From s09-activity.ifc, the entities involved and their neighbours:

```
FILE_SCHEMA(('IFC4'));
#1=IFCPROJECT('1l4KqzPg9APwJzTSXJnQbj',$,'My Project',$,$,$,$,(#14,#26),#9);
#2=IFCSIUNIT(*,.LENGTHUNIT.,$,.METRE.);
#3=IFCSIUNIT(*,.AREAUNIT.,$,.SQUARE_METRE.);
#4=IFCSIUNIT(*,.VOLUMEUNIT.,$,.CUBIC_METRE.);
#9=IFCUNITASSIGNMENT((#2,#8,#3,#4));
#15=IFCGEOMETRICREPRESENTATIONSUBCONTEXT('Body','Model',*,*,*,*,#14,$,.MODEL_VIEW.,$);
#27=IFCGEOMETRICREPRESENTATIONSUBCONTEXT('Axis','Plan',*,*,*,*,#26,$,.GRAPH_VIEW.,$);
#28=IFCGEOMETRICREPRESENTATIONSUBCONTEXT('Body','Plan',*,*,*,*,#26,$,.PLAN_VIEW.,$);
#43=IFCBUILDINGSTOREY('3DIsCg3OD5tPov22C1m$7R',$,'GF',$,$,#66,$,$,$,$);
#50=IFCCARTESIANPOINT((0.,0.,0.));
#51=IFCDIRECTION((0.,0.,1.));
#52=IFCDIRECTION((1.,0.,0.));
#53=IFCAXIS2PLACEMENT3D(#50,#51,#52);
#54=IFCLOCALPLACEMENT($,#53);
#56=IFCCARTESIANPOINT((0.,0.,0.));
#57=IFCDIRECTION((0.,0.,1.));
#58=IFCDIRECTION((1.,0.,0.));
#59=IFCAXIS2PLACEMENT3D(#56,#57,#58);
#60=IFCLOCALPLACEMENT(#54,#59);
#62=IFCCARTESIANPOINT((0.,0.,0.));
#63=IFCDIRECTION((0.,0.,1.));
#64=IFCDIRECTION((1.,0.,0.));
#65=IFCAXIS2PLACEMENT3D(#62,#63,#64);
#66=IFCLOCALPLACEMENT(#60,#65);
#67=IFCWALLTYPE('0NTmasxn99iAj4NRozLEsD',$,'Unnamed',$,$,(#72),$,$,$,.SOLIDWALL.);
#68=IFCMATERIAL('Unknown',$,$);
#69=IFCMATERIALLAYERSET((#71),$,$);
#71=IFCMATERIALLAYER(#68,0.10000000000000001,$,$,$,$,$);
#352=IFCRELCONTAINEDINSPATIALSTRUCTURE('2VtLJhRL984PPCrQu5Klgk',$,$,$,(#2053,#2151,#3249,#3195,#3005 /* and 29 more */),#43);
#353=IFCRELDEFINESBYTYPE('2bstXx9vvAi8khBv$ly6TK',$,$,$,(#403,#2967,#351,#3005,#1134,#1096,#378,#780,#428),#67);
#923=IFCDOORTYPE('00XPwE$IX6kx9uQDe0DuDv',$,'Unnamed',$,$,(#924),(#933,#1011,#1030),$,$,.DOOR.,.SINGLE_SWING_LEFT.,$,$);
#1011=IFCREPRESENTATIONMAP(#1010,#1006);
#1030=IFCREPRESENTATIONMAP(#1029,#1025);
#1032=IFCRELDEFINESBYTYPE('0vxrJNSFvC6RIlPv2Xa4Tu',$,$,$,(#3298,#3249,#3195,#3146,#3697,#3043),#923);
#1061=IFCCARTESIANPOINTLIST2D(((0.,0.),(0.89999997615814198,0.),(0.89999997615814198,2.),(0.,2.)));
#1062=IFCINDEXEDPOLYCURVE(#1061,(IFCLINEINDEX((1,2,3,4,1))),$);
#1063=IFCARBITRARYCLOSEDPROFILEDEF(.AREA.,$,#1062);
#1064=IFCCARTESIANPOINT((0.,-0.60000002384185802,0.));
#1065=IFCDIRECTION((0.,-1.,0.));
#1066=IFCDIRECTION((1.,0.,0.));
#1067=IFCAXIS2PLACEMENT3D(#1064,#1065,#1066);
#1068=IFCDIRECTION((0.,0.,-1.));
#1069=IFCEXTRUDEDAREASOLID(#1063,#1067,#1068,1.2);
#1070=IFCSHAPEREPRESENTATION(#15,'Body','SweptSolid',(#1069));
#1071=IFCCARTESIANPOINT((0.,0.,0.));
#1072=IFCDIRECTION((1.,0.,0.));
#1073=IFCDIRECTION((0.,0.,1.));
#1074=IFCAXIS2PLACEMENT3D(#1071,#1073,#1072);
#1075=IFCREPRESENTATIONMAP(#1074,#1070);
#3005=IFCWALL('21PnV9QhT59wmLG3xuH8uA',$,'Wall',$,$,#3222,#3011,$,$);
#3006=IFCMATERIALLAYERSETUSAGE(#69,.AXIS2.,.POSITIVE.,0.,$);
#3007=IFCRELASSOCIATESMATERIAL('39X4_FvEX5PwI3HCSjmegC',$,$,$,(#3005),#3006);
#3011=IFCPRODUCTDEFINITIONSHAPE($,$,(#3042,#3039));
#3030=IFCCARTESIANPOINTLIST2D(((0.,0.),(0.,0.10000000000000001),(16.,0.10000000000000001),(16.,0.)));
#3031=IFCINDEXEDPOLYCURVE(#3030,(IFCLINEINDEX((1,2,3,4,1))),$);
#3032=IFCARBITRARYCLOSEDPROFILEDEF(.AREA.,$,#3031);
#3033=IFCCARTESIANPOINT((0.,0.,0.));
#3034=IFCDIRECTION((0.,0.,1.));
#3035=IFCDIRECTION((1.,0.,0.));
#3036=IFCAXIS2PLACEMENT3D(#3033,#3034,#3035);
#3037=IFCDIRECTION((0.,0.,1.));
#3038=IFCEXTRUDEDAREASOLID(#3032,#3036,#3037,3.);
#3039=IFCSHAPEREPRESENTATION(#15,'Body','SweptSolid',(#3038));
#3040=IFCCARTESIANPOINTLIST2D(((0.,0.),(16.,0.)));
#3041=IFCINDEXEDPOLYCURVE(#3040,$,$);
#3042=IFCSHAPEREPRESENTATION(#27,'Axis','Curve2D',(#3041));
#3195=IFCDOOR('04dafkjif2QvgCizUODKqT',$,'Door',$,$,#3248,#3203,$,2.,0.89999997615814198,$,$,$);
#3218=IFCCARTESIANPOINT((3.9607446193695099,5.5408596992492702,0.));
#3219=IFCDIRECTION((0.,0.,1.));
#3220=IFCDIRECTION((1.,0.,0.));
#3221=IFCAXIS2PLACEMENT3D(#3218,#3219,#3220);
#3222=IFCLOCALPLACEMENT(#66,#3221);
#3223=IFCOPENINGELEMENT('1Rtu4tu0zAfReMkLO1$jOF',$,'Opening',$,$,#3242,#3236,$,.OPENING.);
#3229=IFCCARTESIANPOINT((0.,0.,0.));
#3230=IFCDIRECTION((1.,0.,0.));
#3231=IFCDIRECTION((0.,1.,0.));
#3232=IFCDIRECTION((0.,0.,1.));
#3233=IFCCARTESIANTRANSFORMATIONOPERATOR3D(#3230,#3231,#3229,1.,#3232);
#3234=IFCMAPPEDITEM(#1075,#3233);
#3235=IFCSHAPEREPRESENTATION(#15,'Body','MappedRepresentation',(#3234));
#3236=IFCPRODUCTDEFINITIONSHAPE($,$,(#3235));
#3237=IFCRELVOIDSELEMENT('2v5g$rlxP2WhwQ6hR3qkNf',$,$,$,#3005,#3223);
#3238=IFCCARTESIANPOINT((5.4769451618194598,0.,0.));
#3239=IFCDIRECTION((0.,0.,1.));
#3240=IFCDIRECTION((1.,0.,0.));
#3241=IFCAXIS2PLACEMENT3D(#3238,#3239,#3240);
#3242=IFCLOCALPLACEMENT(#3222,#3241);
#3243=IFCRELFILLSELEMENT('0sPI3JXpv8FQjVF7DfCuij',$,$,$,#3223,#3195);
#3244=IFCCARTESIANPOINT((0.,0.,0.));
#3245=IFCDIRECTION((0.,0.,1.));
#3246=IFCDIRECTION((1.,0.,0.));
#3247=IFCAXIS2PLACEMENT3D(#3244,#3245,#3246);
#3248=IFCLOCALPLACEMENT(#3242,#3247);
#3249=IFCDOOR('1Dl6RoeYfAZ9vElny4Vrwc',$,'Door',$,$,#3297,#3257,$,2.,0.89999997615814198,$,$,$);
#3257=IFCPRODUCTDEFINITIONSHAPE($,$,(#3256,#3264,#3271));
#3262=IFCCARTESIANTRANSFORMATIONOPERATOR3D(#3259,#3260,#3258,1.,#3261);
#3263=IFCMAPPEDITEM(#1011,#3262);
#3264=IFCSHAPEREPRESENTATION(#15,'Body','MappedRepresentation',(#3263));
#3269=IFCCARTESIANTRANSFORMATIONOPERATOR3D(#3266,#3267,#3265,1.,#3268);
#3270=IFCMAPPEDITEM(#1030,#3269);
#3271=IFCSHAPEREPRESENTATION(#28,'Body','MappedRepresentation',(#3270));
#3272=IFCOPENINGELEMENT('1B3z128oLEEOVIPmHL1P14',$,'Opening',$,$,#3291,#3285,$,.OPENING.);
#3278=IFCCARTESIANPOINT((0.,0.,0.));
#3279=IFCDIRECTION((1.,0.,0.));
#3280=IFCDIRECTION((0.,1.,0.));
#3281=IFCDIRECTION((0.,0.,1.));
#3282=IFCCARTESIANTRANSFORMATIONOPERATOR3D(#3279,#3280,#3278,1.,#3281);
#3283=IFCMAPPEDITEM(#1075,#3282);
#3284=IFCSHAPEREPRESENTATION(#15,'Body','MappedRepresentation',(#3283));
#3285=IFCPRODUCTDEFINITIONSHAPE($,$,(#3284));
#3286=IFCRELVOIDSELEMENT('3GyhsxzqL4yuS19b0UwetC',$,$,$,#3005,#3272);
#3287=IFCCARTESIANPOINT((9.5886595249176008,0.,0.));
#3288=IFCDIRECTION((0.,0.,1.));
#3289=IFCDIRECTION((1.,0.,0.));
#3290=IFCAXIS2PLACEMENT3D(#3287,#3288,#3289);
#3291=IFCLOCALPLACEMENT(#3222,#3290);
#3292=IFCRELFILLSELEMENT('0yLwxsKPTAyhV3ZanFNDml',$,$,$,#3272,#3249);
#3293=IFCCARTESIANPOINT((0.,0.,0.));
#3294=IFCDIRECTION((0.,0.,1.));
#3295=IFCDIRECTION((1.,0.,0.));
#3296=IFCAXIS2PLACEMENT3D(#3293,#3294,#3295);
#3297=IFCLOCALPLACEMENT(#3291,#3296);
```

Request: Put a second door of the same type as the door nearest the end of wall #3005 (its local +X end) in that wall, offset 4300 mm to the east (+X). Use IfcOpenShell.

```python
import ifcopenshell
import ifcopenshell.api.feature
import ifcopenshell.api.geometry
import ifcopenshell.api.root
import ifcopenshell.geom
import ifcopenshell.util.element
import ifcopenshell.util.placement
import ifcopenshell.util.shape
import ifcopenshell.util.unit

model = ifcopenshell.open("s09-activity.ifc")
unit_scale = ifcopenshell.util.unit.calculate_unit_scale(model)
settings = ifcopenshell.geom.settings()


def volume(element):
    """Net volume in cubic metres, openings subtracted."""
    shape = ifcopenshell.geom.create_shape(settings, element)
    return ifcopenshell.util.shape.get_volume(shape.geometry)


door = model.by_guid("1Dl6RoeYfAZ9vElny4Vrwc")
opening = door.FillsVoids[0].RelatingOpeningElement
wall = opening.VoidsElements[0].RelatingBuildingElement
before = volume(wall)
shift = ifcopenshell.util.placement.get_local_placement(wall.ObjectPlacement)[:3, 0] * 4.3 / unit_scale

# copy_class copies the void relationship, type, container and properties, but no geometry.
new_opening = ifcopenshell.api.root.copy_class(model, product=opening)
new_opening.Representation = ifcopenshell.util.element.copy_deep(
    model, opening.Representation, exclude=["IfcGeometricRepresentationContext", "IfcRepresentationMap"]
)
new_door = ifcopenshell.api.root.copy_class(model, product=door)
new_door.Representation = ifcopenshell.util.element.copy_deep(
    model, door.Representation, exclude=["IfcGeometricRepresentationContext", "IfcRepresentationMap"]
)
ifcopenshell.api.feature.add_filling(model, opening=new_opening, element=new_door)

for old, new in ((opening, new_opening), (door, new_door)):
    matrix = ifcopenshell.util.placement.get_local_placement(old.ObjectPlacement)
    matrix[:3, 3] += shift
    ifcopenshell.api.geometry.edit_object_placement(model, product=new, matrix=matrix, is_si=False)

after = volume(wall)

print(f"wall volume {before:.3f} -> {after:.3f} m3")

model.write("s09-activity-out.ifc")
```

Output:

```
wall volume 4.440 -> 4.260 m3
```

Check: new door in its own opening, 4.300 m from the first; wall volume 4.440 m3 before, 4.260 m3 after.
